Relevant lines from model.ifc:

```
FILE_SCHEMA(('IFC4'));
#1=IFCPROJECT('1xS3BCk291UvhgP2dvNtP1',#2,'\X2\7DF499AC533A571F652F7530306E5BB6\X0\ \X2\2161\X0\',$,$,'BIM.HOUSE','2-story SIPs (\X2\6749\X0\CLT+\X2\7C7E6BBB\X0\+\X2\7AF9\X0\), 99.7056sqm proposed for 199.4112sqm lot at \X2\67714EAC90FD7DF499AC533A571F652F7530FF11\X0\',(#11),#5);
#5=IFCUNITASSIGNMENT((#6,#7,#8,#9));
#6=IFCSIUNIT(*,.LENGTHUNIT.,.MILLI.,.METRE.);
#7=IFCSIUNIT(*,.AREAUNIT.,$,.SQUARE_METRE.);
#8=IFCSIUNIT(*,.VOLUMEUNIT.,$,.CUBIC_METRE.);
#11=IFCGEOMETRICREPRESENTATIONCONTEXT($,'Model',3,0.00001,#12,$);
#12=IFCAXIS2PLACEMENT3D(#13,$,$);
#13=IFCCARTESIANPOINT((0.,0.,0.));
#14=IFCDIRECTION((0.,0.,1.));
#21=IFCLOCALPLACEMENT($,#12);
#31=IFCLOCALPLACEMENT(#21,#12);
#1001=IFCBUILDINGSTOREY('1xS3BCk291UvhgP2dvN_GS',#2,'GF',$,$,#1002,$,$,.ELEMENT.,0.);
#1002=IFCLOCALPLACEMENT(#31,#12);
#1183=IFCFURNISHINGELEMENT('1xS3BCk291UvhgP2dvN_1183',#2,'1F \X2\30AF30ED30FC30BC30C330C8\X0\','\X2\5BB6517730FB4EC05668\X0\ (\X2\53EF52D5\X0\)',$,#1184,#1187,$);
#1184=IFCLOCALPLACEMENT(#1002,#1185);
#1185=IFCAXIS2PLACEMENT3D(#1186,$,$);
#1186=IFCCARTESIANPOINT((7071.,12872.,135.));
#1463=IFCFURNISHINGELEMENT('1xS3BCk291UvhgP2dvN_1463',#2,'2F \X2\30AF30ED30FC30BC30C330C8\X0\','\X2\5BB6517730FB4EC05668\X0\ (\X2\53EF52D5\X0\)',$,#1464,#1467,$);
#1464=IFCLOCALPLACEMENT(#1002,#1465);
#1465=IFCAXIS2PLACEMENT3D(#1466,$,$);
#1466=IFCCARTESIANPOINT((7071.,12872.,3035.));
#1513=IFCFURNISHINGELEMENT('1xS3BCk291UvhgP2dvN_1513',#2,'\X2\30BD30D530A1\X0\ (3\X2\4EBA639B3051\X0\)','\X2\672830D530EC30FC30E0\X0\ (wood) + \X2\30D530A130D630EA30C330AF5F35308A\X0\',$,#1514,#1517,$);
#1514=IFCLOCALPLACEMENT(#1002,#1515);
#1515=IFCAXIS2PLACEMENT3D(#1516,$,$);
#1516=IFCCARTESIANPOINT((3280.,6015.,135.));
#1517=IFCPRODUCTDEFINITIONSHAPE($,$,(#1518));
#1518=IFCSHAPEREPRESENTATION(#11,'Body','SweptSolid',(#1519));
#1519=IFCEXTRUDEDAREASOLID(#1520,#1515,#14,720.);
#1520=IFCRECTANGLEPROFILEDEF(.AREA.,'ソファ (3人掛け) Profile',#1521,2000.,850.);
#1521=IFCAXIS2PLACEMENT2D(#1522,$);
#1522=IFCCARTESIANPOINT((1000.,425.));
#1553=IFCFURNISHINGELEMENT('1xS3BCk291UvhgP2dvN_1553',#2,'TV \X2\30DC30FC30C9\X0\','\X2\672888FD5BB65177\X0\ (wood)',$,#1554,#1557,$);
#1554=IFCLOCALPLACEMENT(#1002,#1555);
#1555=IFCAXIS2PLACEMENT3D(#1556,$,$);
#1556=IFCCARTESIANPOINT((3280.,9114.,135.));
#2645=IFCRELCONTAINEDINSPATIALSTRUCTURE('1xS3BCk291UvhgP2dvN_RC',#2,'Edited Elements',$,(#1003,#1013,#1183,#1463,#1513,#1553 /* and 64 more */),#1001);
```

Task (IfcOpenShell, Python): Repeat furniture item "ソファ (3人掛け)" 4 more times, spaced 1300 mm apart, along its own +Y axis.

```python
import ifcopenshell
import ifcopenshell.api.geometry
import ifcopenshell.api.root
import ifcopenshell.util.element
import ifcopenshell.util.placement

model = ifcopenshell.open("model.ifc")


def reuse_history(source, copy):
    """copy_class also copies each property set's owner history, people and application; keep the originals."""
    for rel in copy.IsDefinedBy:
        if rel.is_a("IfcRelDefinesByProperties") and (history := rel.RelatingPropertyDefinition.OwnerHistory):
            rel.RelatingPropertyDefinition.OwnerHistory = source.OwnerHistory
            ifcopenshell.util.element.remove_deep2(model, history)


source = model.by_guid("1xS3BCk291UvhgP2dvN_1513")
base = ifcopenshell.util.placement.get_local_placement(source.ObjectPlacement)
step = base[:3, 1] * 1300.0

for i in range(1, 5):
    copy = ifcopenshell.api.root.copy_class(model, product=source)
    copy.Representation = ifcopenshell.util.element.copy_deep(
        model, source.Representation, exclude=["IfcGeometricRepresentationContext", "IfcRepresentationMap"]
    )
    reuse_history(source, copy)
    matrix = base.copy()
    matrix[:3, 3] += i * step
    print("added at", matrix[:3, 3].round(3) + 0.0)
    ifcopenshell.api.geometry.edit_object_placement(model, product=copy, matrix=matrix, is_si=False)

model.write("model_edited.ifc")
```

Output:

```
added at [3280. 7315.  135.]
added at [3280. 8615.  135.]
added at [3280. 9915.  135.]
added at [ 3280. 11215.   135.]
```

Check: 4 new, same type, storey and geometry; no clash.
